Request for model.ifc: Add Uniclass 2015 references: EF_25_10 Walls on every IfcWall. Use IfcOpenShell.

First a look at what the model holds.

```python
import ifcopenshell

model = ifcopenshell.open("model.ifc")
print(model.schema)
print("classifications:", [c.Name for c in model.by_type("IfcClassification")])
for ifc_class in ("IfcDoor", "IfcRoof", "IfcStair", "IfcWall", "IfcWindow"):
    print(ifc_class, len(model.by_type(ifc_class)))
```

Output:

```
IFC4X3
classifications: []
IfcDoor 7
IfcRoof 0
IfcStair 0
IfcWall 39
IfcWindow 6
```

```python
import ifcopenshell
import ifcopenshell.api.classification

model = ifcopenshell.open("model.ifc")

system = ifcopenshell.api.classification.add_classification(model, classification="Uniclass 2015")

codes = {
    "IfcWall": ("EF_25_10", "Walls"),
}
for ifc_class, (code, name) in codes.items():
    products = model.by_type(ifc_class)
    ifcopenshell.api.classification.add_reference(
        model, products=products, classification=system, identification=code, name=name
    )
    print(code, len(products))

model.write("model-out.ifc")
```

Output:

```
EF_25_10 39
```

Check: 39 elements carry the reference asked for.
